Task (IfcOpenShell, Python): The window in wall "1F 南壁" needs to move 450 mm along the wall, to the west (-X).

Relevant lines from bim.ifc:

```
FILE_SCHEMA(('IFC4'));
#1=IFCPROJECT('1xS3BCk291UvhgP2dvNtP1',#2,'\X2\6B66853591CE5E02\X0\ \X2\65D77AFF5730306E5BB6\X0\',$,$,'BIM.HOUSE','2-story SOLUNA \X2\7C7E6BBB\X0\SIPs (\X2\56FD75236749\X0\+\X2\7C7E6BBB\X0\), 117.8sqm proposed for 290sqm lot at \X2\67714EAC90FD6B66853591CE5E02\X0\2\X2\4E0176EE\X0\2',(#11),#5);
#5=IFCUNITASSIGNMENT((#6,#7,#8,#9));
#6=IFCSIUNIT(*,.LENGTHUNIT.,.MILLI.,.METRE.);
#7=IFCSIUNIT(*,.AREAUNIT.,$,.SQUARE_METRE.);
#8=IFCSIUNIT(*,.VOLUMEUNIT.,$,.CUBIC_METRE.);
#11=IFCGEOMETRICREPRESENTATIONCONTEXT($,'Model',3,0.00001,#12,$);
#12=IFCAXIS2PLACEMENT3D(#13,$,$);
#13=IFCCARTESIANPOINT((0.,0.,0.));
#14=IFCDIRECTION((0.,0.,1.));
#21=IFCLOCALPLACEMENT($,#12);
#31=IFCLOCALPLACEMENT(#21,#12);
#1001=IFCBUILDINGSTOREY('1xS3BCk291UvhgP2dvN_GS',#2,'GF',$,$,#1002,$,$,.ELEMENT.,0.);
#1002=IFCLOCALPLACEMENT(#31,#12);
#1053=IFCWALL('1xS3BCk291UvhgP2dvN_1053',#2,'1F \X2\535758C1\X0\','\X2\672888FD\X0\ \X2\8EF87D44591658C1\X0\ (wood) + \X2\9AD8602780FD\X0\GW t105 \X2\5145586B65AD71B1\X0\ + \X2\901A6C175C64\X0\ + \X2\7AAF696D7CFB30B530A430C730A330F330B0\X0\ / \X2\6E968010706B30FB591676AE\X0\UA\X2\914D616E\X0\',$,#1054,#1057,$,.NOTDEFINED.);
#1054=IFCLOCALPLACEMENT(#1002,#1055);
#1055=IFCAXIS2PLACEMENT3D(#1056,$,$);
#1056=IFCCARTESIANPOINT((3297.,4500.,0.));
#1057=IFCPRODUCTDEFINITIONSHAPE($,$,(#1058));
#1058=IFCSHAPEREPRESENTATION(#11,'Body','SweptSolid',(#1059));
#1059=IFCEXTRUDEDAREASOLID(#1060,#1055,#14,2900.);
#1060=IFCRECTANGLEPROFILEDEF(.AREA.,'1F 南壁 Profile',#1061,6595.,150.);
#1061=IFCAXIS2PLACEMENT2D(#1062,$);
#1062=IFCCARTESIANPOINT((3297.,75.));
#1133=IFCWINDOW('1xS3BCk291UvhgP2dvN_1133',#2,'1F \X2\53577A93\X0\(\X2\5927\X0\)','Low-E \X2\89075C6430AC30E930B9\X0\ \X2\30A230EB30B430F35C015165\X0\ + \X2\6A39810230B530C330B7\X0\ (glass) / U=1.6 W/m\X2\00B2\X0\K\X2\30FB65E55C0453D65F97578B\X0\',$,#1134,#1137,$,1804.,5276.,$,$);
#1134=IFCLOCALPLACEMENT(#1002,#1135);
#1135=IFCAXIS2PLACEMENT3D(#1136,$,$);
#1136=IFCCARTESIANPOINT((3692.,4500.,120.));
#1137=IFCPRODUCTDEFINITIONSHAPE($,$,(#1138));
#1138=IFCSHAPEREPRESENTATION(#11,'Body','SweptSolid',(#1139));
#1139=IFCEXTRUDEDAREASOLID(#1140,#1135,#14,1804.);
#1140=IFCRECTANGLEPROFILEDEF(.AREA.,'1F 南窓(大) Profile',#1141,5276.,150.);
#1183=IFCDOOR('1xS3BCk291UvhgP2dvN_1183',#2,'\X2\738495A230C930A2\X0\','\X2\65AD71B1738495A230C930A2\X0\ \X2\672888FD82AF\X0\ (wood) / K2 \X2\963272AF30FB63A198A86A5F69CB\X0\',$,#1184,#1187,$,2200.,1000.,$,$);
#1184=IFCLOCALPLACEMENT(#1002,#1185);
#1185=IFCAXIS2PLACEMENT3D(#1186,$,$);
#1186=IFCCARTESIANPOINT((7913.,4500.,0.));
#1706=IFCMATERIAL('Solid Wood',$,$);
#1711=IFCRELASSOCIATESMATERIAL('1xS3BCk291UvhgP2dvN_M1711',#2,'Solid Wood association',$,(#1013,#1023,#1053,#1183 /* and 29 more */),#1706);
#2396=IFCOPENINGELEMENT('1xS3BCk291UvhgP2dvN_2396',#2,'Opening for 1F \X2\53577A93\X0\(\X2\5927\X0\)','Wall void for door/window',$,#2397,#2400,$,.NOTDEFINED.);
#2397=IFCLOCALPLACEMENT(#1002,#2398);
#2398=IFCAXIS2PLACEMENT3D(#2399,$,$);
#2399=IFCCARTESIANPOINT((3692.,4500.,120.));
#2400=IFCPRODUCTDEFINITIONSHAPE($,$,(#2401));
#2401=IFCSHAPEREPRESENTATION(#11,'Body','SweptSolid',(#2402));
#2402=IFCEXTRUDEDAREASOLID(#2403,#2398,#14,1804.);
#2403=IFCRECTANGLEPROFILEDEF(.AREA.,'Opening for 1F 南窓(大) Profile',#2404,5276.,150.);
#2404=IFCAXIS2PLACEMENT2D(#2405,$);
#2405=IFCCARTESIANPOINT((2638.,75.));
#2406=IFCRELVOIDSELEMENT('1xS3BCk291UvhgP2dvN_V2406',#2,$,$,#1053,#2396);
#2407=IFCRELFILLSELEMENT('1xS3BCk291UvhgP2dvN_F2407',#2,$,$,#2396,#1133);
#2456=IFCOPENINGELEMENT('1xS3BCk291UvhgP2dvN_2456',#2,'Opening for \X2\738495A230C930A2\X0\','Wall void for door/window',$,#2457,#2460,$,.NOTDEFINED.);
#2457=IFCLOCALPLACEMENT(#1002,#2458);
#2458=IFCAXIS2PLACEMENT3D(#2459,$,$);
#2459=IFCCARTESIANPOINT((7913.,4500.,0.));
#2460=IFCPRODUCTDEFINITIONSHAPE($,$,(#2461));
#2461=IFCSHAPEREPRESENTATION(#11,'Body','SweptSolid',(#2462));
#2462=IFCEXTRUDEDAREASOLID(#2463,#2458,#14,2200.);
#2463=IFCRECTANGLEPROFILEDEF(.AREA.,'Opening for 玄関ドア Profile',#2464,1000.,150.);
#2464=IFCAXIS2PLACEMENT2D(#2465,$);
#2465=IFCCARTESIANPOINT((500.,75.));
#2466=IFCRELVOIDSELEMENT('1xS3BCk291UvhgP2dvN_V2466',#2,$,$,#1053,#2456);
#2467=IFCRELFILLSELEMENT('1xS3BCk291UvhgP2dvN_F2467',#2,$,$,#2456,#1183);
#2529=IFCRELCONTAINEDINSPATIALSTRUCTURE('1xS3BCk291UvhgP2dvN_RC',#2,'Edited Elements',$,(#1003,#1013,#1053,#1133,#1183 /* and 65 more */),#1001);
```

```python
import ifcopenshell
import ifcopenshell.api.geometry
import ifcopenshell.util.placement

model = ifcopenshell.open("bim.ifc")

window = model.by_guid("1xS3BCk291UvhgP2dvN_1133")
opening = window.FillsVoids[0].RelatingOpeningElement
wall = opening.VoidsElements[0].RelatingBuildingElement

wall_matrix = ifcopenshell.util.placement.get_local_placement(wall.ObjectPlacement)
shift = wall_matrix[:3, 0] * -450.0
before = ifcopenshell.util.placement.get_local_placement(window.ObjectPlacement)[:3, 3].copy()

# The window is not placed relative to its opening, so move both.
for product in (opening, window):
    matrix = ifcopenshell.util.placement.get_local_placement(product.ObjectPlacement)
    matrix[:3, 3] += shift
    ifcopenshell.api.geometry.edit_object_placement(model, product=product, matrix=matrix, is_si=False)

after = ifcopenshell.util.placement.get_local_placement(window.ObjectPlacement)[:3, 3]
print("window moved by", (after - before).round(3) + 0.0)

model.write("bim_rev.ifc")
```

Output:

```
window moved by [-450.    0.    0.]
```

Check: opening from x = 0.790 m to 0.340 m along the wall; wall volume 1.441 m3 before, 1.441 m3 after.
